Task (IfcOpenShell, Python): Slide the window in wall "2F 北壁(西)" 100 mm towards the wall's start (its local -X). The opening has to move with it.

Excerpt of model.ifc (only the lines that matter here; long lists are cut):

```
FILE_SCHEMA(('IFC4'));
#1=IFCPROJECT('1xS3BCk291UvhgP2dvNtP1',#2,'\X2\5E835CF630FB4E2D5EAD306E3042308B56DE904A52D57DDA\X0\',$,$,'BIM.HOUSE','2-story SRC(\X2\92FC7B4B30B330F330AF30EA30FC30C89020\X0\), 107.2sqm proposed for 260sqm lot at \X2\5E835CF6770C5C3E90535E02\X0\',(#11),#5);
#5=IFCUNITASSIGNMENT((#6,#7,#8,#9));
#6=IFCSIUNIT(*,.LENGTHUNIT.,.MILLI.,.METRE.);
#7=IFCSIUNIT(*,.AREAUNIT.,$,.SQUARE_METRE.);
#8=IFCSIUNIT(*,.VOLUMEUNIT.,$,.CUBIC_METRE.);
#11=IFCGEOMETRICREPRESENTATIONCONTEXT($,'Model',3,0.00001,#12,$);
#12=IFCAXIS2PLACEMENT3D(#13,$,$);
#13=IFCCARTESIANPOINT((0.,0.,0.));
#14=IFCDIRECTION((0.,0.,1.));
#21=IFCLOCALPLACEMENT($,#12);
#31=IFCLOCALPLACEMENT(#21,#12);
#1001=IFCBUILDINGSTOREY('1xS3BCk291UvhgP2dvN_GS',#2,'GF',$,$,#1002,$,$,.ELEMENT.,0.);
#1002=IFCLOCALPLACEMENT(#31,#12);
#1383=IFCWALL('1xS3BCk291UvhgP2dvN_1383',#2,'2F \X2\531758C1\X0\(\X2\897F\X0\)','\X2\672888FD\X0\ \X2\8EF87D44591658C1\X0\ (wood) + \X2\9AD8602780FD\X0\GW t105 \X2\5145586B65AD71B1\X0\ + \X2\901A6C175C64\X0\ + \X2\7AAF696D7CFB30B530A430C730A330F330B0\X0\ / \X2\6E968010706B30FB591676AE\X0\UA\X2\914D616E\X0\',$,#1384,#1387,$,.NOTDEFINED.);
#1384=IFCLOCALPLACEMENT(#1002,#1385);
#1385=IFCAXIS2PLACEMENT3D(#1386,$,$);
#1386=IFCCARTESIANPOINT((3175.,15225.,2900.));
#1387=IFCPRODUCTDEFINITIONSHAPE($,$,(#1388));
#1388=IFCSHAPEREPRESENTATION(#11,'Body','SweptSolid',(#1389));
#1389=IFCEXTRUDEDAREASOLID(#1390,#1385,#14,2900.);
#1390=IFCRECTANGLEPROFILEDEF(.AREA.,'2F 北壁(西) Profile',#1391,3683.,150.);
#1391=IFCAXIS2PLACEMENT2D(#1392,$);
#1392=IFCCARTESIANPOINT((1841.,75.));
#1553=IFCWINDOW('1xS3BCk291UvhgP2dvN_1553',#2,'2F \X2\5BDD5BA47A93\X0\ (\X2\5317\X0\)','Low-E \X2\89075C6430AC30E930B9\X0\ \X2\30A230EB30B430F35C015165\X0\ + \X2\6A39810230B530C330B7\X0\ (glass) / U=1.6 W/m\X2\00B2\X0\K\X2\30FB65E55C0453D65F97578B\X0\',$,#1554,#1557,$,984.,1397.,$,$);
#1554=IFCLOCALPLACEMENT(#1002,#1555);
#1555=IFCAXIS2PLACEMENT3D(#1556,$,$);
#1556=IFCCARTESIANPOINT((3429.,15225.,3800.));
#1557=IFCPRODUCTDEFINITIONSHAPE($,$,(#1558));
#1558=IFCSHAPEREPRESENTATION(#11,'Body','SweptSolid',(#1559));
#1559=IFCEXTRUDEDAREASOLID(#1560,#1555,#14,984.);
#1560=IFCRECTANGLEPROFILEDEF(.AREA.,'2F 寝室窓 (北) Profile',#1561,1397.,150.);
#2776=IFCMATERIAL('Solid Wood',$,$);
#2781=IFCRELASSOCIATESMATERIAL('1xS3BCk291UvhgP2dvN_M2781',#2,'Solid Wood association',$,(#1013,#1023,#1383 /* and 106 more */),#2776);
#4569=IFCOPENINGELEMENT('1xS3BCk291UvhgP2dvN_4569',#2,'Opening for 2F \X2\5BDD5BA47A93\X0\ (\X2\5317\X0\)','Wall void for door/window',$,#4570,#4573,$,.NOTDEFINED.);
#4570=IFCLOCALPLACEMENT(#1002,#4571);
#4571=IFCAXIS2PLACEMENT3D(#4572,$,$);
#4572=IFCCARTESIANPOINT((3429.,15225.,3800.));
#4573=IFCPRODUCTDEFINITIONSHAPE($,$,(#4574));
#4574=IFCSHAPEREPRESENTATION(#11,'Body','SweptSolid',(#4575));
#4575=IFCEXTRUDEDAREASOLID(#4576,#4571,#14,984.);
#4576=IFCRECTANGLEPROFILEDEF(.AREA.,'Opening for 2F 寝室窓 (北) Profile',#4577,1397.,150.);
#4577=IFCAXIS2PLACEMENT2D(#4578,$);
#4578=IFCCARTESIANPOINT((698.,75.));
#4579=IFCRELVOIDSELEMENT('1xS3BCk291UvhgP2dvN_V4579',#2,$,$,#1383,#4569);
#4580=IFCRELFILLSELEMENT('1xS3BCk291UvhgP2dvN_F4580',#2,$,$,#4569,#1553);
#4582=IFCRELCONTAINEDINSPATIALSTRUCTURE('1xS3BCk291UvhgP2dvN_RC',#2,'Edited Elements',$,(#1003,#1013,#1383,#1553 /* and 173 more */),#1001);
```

```python
import ifcopenshell
import ifcopenshell.api.geometry
import ifcopenshell.util.placement

model = ifcopenshell.open("model.ifc")

window = model.by_guid("1xS3BCk291UvhgP2dvN_1553")
opening = window.FillsVoids[0].RelatingOpeningElement
wall = opening.VoidsElements[0].RelatingBuildingElement

wall_matrix = ifcopenshell.util.placement.get_local_placement(wall.ObjectPlacement)
shift = wall_matrix[:3, 0] * -100.0
before = ifcopenshell.util.placement.get_local_placement(window.ObjectPlacement)[:3, 3].copy()

# The window is not placed relative to its opening, so move both.
for product in (opening, window):
    matrix = ifcopenshell.util.placement.get_local_placement(product.ObjectPlacement)
    matrix[:3, 3] += shift
    ifcopenshell.api.geometry.edit_object_placement(model, product=product, matrix=matrix, is_si=False)

after = ifcopenshell.util.placement.get_local_placement(window.ObjectPlacement)[:3, 3]
print("window moved by", (after - before).round(3) + 0.0)

model.write("model_v2.ifc")
```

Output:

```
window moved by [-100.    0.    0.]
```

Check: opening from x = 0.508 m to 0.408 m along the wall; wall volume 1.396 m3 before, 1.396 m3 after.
